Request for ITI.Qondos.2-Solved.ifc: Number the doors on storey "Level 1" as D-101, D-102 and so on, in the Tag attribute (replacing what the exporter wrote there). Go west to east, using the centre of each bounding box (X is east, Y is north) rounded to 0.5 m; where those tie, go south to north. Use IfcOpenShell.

First a look at what the model holds.

```python
import ifcopenshell
import ifcopenshell.util.element
import ifcopenshell.util.placement

model = ifcopenshell.open("ITI.Qondos.2-Solved.ifc")
print(model.schema)
storey = next(s for s in model.by_type("IfcBuildingStorey") if s.Name == "Level 1")
doors = [e for e in ifcopenshell.util.element.get_decomposition(storey) if e.is_a("IfcDoor")]
for e in sorted(doors, key=lambda e: e.id()):
    origin = ifcopenshell.util.placement.get_local_placement(e.ObjectPlacement)[:3, 3]
    print(e.id(), e.Tag, e.Name, origin.round(2) + 0.0, sep=" | ")
```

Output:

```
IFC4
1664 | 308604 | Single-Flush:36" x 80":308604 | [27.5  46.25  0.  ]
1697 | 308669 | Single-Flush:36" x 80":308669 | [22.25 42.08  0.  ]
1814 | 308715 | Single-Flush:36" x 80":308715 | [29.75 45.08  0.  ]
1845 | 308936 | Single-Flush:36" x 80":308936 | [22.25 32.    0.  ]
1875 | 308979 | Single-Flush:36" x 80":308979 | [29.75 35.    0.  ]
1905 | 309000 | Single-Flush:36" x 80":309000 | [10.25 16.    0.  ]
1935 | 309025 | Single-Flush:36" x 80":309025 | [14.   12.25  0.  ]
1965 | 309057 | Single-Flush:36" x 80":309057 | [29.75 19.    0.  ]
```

```python
import ifcopenshell
import ifcopenshell.geom
import ifcopenshell.util.element
import ifcopenshell.util.shape

model = ifcopenshell.open("ITI.Qondos.2-Solved.ifc")
settings = ifcopenshell.geom.settings()
settings.set("use-world-coords", True)


def centre(element):
    shape = ifcopenshell.geom.create_shape(settings, element)
    return ifcopenshell.util.shape.get_bbox_centroid(shape.geometry)


storey = next(s for s in model.by_type("IfcBuildingStorey") if s.Name == "Level 1")
doors = [e for e in ifcopenshell.util.element.get_decomposition(storey) if e.is_a("IfcDoor")]

# Insertion points can sit at a corner or the storey origin, so sort by the geometry (in metres).
centres = {e: centre(e) for e in doors}
doors.sort(key=lambda e: (round(centres[e][0] / 0.5), centres[e][1]))

for i, e in enumerate(doors, start=1):
    number = f"D-1{i:02d}"
    e.Tag = number
    print(e.id(), number)

model.write("ITI.Qondos.2-Solved_edited.ifc")
```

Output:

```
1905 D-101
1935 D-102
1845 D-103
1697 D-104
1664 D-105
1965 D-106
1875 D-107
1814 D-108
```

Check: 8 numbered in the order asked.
